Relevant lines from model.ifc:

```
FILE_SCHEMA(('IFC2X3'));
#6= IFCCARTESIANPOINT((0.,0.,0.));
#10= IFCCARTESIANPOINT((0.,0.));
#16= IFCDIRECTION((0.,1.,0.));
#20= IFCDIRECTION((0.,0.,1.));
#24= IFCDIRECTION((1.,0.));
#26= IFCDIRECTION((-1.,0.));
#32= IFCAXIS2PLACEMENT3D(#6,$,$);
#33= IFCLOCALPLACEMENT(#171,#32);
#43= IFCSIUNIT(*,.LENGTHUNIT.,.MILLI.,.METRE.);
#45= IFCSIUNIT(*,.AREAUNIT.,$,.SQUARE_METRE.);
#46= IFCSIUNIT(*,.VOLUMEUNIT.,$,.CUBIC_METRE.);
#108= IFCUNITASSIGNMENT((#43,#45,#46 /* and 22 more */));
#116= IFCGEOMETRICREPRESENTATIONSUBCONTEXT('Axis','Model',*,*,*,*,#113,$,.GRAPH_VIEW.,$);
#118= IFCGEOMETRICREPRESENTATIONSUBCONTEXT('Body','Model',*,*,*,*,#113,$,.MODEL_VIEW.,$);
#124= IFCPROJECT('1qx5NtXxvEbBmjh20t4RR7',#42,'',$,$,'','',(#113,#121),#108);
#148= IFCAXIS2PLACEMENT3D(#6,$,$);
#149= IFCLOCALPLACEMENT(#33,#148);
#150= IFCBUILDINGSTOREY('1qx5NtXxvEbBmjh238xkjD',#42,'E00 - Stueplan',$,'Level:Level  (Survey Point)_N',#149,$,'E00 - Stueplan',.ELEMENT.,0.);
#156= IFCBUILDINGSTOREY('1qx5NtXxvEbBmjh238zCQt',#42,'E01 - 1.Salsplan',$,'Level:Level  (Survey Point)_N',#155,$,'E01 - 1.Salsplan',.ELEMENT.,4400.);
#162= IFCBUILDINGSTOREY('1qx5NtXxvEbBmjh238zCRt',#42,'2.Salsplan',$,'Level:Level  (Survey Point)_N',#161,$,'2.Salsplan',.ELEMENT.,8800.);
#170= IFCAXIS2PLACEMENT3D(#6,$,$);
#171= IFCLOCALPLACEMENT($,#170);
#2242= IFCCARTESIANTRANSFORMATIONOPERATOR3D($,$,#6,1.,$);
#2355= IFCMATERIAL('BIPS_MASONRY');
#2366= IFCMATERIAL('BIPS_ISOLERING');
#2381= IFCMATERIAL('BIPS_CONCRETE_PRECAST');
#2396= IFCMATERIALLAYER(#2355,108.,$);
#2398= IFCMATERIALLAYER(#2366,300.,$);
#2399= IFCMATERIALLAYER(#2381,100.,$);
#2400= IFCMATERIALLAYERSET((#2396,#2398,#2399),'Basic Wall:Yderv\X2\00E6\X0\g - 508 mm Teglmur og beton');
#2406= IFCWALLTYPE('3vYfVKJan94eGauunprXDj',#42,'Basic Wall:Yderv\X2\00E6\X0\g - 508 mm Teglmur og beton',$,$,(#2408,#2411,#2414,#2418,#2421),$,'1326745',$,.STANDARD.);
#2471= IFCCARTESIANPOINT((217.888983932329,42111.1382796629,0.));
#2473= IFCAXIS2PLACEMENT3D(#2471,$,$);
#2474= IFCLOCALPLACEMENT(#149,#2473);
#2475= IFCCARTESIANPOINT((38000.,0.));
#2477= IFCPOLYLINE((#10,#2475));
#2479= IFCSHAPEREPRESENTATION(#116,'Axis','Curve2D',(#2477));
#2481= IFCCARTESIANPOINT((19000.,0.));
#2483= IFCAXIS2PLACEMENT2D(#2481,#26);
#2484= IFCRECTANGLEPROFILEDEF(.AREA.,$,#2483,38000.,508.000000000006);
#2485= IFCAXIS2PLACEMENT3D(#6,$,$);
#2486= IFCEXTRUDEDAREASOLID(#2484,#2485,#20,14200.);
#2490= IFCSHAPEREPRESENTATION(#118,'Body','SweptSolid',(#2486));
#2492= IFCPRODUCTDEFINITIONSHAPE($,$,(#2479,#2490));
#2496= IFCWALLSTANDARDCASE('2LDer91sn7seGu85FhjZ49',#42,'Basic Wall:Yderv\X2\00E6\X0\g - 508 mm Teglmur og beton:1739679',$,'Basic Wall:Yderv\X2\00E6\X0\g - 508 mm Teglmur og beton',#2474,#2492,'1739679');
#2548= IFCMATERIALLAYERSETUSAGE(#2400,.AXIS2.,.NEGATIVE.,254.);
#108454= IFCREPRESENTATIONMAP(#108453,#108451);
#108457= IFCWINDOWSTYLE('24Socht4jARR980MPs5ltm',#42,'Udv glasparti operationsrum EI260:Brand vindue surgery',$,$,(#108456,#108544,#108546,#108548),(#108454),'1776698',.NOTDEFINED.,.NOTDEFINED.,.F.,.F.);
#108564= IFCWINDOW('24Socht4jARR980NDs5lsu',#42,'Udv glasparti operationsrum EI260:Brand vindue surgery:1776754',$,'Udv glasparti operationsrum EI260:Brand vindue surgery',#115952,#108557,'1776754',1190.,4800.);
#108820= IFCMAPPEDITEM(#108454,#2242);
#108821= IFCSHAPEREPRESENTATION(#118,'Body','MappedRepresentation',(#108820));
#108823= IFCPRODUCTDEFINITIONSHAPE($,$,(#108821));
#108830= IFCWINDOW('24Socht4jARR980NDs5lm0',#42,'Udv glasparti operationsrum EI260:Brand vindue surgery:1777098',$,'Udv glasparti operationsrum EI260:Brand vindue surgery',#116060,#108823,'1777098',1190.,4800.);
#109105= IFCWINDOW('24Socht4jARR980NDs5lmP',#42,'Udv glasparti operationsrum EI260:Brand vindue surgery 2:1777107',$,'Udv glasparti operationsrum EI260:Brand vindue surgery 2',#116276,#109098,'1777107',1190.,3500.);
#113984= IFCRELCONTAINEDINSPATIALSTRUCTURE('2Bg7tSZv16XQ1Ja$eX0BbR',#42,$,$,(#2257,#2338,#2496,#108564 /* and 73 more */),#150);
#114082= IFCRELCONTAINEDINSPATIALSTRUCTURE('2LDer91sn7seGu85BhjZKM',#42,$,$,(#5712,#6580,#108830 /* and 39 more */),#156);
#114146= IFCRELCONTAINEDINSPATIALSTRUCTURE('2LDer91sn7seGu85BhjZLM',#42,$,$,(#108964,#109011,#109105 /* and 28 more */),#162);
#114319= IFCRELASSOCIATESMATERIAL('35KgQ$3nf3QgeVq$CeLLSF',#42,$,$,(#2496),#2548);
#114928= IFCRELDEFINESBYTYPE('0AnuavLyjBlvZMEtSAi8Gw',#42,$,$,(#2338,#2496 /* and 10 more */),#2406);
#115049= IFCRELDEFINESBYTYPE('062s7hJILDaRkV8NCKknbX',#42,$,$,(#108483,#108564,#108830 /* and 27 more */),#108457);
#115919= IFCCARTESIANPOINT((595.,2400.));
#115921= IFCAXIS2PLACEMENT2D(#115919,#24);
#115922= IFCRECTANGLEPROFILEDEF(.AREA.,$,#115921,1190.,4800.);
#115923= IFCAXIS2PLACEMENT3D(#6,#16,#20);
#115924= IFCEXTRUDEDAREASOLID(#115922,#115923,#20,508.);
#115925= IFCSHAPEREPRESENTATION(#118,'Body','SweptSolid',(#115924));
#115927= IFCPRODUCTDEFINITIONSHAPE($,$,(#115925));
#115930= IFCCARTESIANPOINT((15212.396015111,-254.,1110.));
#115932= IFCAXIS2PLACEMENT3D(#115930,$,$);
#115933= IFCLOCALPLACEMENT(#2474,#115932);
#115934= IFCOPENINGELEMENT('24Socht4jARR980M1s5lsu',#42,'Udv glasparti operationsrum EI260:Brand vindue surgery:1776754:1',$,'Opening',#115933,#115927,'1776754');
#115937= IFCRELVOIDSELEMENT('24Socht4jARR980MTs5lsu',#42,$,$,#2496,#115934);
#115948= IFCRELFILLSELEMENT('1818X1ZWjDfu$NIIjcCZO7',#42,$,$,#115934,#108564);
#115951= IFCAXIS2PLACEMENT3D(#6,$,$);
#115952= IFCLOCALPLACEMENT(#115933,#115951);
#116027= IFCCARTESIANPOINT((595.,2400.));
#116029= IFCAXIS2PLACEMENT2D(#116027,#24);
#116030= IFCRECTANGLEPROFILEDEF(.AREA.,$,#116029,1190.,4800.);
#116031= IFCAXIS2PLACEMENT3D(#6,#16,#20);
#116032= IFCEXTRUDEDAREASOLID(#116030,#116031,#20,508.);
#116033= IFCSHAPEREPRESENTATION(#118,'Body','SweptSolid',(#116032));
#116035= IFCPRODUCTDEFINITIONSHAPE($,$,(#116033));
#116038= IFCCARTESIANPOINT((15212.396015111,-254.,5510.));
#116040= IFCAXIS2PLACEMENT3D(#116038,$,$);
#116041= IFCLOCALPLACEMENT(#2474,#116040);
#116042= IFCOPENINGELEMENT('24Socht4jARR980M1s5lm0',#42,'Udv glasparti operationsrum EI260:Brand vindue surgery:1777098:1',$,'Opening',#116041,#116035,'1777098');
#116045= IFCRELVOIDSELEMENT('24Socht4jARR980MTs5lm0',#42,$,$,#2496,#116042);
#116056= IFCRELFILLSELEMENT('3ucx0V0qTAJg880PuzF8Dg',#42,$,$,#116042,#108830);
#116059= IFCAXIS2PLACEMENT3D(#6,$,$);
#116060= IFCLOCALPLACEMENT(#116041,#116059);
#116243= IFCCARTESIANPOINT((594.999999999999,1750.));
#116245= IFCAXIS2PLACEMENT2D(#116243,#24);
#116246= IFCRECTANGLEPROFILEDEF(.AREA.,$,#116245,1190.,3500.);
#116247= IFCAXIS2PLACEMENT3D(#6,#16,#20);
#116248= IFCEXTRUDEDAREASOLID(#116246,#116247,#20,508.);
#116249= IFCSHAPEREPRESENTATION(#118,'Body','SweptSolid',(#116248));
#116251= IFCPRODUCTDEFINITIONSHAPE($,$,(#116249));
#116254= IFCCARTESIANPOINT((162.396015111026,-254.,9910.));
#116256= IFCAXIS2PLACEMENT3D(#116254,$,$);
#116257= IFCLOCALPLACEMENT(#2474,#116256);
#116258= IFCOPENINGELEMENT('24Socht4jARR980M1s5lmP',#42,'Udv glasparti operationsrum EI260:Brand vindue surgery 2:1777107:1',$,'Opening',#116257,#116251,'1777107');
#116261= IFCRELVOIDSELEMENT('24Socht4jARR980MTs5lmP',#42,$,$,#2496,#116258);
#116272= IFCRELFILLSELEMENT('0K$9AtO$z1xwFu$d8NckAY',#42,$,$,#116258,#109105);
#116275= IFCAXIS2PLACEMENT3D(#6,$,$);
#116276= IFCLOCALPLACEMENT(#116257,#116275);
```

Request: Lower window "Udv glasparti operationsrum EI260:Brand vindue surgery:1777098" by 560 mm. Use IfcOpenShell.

```python
import numpy as np
import ifcopenshell
import ifcopenshell.api.geometry
import ifcopenshell.util.placement
import ifcopenshell.util.unit

model = ifcopenshell.open("model.ifc")
unit_scale = ifcopenshell.util.unit.calculate_unit_scale(model)

window = model.by_guid("24Socht4jARR980NDs5lm0")
opening = window.FillsVoids[0].RelatingOpeningElement
dz = -560.0

shift = np.array([0.0, 0.0, dz])
# The window is placed relative to its opening, so it follows when the opening moves.
matrix = ifcopenshell.util.placement.get_local_placement(opening.ObjectPlacement)
matrix[:3, 3] += shift
ifcopenshell.api.geometry.edit_object_placement(
    model, product=opening, matrix=matrix, is_si=False, should_transform_children=True
)

print(f"moved by {dz * unit_scale:+.3f} m")

model.write("model_v2.ifc")
```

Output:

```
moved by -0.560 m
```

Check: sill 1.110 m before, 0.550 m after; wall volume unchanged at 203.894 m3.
